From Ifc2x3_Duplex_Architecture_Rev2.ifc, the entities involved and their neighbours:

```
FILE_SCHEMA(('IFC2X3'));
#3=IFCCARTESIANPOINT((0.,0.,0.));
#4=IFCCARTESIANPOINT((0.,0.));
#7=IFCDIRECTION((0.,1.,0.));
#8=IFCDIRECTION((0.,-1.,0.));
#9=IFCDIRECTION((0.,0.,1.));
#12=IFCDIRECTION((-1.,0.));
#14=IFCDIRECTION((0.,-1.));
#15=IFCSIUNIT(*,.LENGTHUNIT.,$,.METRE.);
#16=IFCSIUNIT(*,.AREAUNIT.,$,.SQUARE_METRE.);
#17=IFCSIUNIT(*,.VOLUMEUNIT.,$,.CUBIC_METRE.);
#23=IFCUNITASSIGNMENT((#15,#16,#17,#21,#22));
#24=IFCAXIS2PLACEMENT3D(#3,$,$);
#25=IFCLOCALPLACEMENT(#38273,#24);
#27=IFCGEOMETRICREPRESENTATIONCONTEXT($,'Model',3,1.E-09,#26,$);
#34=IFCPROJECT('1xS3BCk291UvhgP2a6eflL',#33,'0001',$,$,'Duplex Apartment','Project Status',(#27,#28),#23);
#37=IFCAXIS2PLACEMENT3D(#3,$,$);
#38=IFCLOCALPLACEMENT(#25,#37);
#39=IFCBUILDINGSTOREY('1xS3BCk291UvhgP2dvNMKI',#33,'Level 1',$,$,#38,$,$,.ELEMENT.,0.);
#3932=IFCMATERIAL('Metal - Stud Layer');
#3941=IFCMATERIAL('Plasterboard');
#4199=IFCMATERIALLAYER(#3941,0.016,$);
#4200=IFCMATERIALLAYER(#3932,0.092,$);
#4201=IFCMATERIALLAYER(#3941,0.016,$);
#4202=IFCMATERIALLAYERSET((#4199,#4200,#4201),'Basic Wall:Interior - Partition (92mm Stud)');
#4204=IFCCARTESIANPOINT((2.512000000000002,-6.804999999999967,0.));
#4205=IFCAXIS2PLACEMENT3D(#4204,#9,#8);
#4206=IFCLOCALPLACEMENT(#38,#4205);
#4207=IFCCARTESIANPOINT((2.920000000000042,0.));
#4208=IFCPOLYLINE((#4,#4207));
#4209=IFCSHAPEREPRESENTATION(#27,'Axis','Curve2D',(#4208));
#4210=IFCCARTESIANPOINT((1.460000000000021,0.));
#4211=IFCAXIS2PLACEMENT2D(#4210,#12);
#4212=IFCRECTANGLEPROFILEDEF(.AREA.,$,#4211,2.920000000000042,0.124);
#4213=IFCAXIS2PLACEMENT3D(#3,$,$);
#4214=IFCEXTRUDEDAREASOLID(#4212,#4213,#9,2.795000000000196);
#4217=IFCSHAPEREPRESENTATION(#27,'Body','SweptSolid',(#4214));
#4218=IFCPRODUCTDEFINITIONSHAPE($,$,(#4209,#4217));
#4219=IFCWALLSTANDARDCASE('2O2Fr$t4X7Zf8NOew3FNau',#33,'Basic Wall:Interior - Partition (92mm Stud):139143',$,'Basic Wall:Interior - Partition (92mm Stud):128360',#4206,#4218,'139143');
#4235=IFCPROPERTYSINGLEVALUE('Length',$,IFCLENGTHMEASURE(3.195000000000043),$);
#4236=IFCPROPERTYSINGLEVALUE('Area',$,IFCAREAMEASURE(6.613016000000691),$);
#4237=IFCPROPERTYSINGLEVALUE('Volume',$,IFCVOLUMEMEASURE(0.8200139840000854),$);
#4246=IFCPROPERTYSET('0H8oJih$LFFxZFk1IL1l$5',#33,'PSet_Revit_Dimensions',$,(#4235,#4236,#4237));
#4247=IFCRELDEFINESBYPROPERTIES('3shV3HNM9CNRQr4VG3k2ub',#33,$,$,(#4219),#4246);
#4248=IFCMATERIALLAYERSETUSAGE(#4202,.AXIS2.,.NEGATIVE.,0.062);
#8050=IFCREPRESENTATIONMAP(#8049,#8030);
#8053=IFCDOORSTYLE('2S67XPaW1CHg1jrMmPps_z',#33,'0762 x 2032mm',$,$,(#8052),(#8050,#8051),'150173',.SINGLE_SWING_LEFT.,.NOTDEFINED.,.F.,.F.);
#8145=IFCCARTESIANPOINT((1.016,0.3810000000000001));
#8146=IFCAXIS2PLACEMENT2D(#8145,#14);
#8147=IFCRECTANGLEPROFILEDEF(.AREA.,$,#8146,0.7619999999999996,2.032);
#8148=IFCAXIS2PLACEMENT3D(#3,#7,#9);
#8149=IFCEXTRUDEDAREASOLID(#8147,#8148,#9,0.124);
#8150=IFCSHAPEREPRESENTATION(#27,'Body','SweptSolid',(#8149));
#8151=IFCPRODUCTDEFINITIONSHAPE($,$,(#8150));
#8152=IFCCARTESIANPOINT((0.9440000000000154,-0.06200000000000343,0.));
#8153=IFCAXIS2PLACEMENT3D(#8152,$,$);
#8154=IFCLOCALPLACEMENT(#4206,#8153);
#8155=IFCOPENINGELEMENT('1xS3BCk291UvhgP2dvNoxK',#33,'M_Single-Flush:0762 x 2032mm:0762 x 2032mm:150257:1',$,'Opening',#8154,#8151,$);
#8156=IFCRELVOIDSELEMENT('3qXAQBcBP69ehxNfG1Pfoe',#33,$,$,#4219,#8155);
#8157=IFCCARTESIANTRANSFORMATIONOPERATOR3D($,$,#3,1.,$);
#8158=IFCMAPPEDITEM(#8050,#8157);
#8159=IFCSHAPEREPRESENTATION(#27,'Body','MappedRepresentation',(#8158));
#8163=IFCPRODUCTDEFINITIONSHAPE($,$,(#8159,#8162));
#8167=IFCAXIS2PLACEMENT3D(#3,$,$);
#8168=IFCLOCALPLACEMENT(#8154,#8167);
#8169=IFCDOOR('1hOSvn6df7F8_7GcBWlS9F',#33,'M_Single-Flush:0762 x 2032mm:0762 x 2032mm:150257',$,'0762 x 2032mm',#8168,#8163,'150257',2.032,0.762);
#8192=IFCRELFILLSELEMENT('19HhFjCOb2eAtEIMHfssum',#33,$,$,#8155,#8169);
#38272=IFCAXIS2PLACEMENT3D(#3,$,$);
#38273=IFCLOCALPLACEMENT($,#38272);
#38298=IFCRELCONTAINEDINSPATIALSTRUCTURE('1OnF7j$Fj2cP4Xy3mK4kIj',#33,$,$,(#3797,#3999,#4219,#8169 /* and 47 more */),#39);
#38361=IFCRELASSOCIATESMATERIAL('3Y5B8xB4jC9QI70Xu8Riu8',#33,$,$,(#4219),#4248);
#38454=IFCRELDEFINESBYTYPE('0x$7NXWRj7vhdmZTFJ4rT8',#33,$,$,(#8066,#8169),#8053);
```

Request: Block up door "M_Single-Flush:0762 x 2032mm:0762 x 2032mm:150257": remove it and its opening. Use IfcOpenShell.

```python
import ifcopenshell
import ifcopenshell.api.feature
import ifcopenshell.api.pset
import ifcopenshell.api.root
import ifcopenshell.geom
import ifcopenshell.util.element
import ifcopenshell.util.shape
import ifcopenshell.util.unit

model = ifcopenshell.open("Ifc2x3_Duplex_Architecture_Rev2.ifc")
area_scale = ifcopenshell.util.unit.calculate_unit_scale(model, "AREAUNIT")
volume_scale = ifcopenshell.util.unit.calculate_unit_scale(model, "VOLUMEUNIT")
settings = ifcopenshell.geom.settings()


def volume(element):
    """Net volume in cubic metres, openings subtracted."""
    shape = ifcopenshell.geom.create_shape(settings, element)
    return ifcopenshell.util.shape.get_volume(shape.geometry)


door = model.by_guid("1hOSvn6df7F8_7GcBWlS9F")
opening = door.FillsVoids[0].RelatingOpeningElement
wall = opening.VoidsElements[0].RelatingBuildingElement
before = volume(wall)

ifcopenshell.api.root.remove_product(model, product=door)
ifcopenshell.api.feature.remove_feature(model, feature=opening)

after = volume(wall)
thickness = 0.124  # wall thickness in metres

# Update the wall's stored quantities.
pset = model.by_id(ifcopenshell.util.element.get_pset(wall, "PSet_Revit_Dimensions", should_inherit=False)["id"])
ifcopenshell.api.pset.edit_pset(model, pset=pset, properties={
    "Area": model.create_entity("IfcAreaMeasure", after / thickness / area_scale),
    "Volume": model.create_entity("IfcVolumeMeasure", after / volume_scale),
})

print(f"wall volume {before:.3f} -> {after:.3f} m3")

model.write("Ifc2x3_Duplex_Architecture_Rev2-out.ifc")
```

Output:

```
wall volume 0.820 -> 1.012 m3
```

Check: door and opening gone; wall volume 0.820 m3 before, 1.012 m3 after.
